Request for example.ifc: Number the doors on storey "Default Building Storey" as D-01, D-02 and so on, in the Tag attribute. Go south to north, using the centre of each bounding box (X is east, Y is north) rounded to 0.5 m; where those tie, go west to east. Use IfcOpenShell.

First a look at what the model holds.

```python
import ifcopenshell
import ifcopenshell.util.element
import ifcopenshell.util.placement

model = ifcopenshell.open("example.ifc")
print(model.schema)
storey = next(s for s in model.by_type("IfcBuildingStorey") if s.Name == "Default Building Storey")
doors = [e for e in ifcopenshell.util.element.get_decomposition(storey) if e.is_a("IfcDoor")]
for e in sorted(doors, key=lambda e: e.id()):
    origin = ifcopenshell.util.placement.get_local_placement(e.ObjectPlacement)[:3, 3]
    print(e.id(), e.Tag, e.Name, origin.round(2) + 0.0, sep=" | ")
```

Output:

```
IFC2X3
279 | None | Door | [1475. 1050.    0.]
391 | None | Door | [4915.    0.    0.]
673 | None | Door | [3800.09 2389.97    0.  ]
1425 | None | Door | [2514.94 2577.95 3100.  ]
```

```python
import ifcopenshell
import ifcopenshell.geom
import ifcopenshell.util.element
import ifcopenshell.util.shape

model = ifcopenshell.open("example.ifc")
settings = ifcopenshell.geom.settings()
settings.set("use-world-coords", True)


def centre(element):
    shape = ifcopenshell.geom.create_shape(settings, element)
    return ifcopenshell.util.shape.get_bbox_centroid(shape.geometry)


storey = next(s for s in model.by_type("IfcBuildingStorey") if s.Name == "Default Building Storey")
doors = [e for e in ifcopenshell.util.element.get_decomposition(storey) if e.is_a("IfcDoor")]

# Insertion points can sit at a corner or the storey origin, so sort by the geometry (in metres).
centres = {e: centre(e) for e in doors}
doors.sort(key=lambda e: (round(centres[e][1] / 0.5), centres[e][0]))

for i, e in enumerate(doors, start=1):
    number = f"D-{i:02d}"
    e.Tag = number
    print(e.id(), number)

model.write("example-out.ifc")
```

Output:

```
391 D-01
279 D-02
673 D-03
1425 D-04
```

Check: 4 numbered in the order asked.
